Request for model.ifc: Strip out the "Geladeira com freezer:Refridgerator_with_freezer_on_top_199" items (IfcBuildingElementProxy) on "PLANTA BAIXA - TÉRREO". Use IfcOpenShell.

First a look at what the model holds.

```python
import ifcopenshell
import ifcopenshell.util.element

model = ifcopenshell.open("model.ifc")
print(model.schema)
storey = next(s for s in model.by_type("IfcBuildingStorey") if s.Name == "PLANTA BAIXA - TÉRREO")
proxies = [e for e in ifcopenshell.util.element.get_decomposition(storey) if e.is_a("IfcBuildingElementProxy")]
seen = {}
for e in proxies:
    element_type = ifcopenshell.util.element.get_type(e)
    name = element_type.Name if element_type not in (None, e) else None
    seen[name] = seen.get(name, 0) + 1
for name, count in sorted(seen.items(), key=str):
    print(count, "x", name)
```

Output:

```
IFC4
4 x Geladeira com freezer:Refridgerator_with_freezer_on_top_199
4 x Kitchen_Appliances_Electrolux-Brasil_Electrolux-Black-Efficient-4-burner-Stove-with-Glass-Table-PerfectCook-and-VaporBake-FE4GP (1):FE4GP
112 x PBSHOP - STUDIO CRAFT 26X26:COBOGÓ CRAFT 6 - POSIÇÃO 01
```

```python
import ifcopenshell
import ifcopenshell.api.root
import ifcopenshell.util.element

model = ifcopenshell.open("model.ifc")

storey = next(s for s in model.by_type("IfcBuildingStorey") if s.Name == "PLANTA BAIXA - TÉRREO")
proxies = [e for e in ifcopenshell.util.element.get_decomposition(storey) if e.is_a("IfcBuildingElementProxy")]
targets = [e for e in proxies if (t := ifcopenshell.util.element.get_type(e)) not in (None, e) and t.Name == "Geladeira com freezer:Refridgerator_with_freezer_on_top_199"]

for e in targets:
    ifcopenshell.api.root.remove_product(model, product=e)
print(len(targets), "removed")

model.write("model_updated.ifc")
```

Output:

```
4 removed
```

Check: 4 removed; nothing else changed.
